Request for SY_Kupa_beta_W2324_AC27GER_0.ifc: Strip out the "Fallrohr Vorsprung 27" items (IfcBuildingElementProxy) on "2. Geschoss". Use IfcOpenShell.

First a look at what the model holds.

```python
import ifcopenshell
import ifcopenshell.util.element

model = ifcopenshell.open("SY_Kupa_beta_W2324_AC27GER_0.ifc")
print(model.schema)
storey = next(s for s in model.by_type("IfcBuildingStorey") if s.Name == "2. Geschoss")
proxies = [e for e in ifcopenshell.util.element.get_decomposition(storey) if e.is_a("IfcBuildingElementProxy")]
seen = {}
for e in proxies:
    element_type = ifcopenshell.util.element.get_type(e)
    name = element_type.Name if element_type not in (None, e) else None
    seen[name] = seen.get(name, 0) + 1
for name, count in sorted(seen.items(), key=str):
    print(count, "x", name)
```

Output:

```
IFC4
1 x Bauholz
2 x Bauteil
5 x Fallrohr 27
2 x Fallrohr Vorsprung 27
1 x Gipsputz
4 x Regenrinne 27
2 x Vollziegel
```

```python
import ifcopenshell
import ifcopenshell.api.root
import ifcopenshell.util.element

model = ifcopenshell.open("SY_Kupa_beta_W2324_AC27GER_0.ifc")

storey = next(s for s in model.by_type("IfcBuildingStorey") if s.Name == "2. Geschoss")
proxies = [e for e in ifcopenshell.util.element.get_decomposition(storey) if e.is_a("IfcBuildingElementProxy")]
targets = [e for e in proxies if (t := ifcopenshell.util.element.get_type(e)) not in (None, e) and t.Name == "Fallrohr Vorsprung 27"]

for e in targets:
    ifcopenshell.api.root.remove_product(model, product=e)
print(len(targets), "removed")

model.write("SY_Kupa_beta_W2324_AC27GER_0_rev.ifc")
```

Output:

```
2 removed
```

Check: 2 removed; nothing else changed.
